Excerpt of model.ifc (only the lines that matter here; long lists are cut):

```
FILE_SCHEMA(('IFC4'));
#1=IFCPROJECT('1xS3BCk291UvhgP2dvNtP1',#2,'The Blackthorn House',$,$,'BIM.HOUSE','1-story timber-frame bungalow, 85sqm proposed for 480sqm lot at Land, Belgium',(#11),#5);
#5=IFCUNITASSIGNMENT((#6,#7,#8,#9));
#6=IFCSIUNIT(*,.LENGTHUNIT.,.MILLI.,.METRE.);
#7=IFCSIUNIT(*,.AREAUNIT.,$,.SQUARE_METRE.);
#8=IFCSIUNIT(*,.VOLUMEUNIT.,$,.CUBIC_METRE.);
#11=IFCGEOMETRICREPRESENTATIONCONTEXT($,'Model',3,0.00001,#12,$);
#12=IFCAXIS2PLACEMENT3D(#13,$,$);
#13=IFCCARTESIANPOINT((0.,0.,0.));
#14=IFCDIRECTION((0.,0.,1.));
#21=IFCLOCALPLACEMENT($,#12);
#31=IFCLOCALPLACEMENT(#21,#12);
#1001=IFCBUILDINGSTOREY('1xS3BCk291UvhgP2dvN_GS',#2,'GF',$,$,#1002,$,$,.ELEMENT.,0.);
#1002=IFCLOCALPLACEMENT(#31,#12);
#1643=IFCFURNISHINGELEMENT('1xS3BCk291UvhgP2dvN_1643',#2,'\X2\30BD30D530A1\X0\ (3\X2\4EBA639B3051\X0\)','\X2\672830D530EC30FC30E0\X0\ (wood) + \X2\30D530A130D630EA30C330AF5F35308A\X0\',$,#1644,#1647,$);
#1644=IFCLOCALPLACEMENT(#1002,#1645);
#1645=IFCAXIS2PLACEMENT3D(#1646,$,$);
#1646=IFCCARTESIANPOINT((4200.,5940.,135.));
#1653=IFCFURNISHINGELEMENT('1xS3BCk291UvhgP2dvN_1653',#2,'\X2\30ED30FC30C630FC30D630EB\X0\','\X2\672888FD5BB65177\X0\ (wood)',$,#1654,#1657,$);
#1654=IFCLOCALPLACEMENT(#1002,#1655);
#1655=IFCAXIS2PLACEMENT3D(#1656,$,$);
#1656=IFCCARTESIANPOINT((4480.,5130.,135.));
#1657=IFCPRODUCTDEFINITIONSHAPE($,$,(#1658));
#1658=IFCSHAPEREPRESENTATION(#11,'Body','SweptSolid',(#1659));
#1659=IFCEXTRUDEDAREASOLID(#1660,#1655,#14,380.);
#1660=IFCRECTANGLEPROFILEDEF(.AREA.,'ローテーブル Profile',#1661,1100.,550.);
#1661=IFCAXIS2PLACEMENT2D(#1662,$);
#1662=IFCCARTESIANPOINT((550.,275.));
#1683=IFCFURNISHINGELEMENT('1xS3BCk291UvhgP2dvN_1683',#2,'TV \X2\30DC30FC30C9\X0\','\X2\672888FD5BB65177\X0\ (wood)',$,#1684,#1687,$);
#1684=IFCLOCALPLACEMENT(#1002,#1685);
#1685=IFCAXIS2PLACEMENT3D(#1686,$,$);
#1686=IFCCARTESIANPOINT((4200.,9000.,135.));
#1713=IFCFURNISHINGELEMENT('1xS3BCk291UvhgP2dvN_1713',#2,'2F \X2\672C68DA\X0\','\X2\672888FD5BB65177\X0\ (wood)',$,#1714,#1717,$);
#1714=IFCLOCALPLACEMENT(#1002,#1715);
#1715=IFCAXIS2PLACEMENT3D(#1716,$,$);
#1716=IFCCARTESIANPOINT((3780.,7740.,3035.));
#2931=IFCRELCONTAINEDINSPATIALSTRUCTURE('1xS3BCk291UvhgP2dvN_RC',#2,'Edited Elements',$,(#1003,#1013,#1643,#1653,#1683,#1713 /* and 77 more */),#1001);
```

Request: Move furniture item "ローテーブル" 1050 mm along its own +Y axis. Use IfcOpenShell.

```python
import ifcopenshell
import ifcopenshell.api.geometry
import ifcopenshell.util.placement
import ifcopenshell.util.unit

model = ifcopenshell.open("model.ifc")
unit_scale = ifcopenshell.util.unit.calculate_unit_scale(model)

item = model.by_guid("1xS3BCk291UvhgP2dvN_1653")
matrix = ifcopenshell.util.placement.get_local_placement(item.ObjectPlacement)
matrix[:3, 3] += matrix[:3, 1] * 1.05 / unit_scale
ifcopenshell.api.geometry.edit_object_placement(model, product=item, matrix=matrix, is_si=False)

print(ifcopenshell.util.placement.get_local_placement(item.ObjectPlacement).round(3) + 0.0)

model.write("model_updated.ifc")
```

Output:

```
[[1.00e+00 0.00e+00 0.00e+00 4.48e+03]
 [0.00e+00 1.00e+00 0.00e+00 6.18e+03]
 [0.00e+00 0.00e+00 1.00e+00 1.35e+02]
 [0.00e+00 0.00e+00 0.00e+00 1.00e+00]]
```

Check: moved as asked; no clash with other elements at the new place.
